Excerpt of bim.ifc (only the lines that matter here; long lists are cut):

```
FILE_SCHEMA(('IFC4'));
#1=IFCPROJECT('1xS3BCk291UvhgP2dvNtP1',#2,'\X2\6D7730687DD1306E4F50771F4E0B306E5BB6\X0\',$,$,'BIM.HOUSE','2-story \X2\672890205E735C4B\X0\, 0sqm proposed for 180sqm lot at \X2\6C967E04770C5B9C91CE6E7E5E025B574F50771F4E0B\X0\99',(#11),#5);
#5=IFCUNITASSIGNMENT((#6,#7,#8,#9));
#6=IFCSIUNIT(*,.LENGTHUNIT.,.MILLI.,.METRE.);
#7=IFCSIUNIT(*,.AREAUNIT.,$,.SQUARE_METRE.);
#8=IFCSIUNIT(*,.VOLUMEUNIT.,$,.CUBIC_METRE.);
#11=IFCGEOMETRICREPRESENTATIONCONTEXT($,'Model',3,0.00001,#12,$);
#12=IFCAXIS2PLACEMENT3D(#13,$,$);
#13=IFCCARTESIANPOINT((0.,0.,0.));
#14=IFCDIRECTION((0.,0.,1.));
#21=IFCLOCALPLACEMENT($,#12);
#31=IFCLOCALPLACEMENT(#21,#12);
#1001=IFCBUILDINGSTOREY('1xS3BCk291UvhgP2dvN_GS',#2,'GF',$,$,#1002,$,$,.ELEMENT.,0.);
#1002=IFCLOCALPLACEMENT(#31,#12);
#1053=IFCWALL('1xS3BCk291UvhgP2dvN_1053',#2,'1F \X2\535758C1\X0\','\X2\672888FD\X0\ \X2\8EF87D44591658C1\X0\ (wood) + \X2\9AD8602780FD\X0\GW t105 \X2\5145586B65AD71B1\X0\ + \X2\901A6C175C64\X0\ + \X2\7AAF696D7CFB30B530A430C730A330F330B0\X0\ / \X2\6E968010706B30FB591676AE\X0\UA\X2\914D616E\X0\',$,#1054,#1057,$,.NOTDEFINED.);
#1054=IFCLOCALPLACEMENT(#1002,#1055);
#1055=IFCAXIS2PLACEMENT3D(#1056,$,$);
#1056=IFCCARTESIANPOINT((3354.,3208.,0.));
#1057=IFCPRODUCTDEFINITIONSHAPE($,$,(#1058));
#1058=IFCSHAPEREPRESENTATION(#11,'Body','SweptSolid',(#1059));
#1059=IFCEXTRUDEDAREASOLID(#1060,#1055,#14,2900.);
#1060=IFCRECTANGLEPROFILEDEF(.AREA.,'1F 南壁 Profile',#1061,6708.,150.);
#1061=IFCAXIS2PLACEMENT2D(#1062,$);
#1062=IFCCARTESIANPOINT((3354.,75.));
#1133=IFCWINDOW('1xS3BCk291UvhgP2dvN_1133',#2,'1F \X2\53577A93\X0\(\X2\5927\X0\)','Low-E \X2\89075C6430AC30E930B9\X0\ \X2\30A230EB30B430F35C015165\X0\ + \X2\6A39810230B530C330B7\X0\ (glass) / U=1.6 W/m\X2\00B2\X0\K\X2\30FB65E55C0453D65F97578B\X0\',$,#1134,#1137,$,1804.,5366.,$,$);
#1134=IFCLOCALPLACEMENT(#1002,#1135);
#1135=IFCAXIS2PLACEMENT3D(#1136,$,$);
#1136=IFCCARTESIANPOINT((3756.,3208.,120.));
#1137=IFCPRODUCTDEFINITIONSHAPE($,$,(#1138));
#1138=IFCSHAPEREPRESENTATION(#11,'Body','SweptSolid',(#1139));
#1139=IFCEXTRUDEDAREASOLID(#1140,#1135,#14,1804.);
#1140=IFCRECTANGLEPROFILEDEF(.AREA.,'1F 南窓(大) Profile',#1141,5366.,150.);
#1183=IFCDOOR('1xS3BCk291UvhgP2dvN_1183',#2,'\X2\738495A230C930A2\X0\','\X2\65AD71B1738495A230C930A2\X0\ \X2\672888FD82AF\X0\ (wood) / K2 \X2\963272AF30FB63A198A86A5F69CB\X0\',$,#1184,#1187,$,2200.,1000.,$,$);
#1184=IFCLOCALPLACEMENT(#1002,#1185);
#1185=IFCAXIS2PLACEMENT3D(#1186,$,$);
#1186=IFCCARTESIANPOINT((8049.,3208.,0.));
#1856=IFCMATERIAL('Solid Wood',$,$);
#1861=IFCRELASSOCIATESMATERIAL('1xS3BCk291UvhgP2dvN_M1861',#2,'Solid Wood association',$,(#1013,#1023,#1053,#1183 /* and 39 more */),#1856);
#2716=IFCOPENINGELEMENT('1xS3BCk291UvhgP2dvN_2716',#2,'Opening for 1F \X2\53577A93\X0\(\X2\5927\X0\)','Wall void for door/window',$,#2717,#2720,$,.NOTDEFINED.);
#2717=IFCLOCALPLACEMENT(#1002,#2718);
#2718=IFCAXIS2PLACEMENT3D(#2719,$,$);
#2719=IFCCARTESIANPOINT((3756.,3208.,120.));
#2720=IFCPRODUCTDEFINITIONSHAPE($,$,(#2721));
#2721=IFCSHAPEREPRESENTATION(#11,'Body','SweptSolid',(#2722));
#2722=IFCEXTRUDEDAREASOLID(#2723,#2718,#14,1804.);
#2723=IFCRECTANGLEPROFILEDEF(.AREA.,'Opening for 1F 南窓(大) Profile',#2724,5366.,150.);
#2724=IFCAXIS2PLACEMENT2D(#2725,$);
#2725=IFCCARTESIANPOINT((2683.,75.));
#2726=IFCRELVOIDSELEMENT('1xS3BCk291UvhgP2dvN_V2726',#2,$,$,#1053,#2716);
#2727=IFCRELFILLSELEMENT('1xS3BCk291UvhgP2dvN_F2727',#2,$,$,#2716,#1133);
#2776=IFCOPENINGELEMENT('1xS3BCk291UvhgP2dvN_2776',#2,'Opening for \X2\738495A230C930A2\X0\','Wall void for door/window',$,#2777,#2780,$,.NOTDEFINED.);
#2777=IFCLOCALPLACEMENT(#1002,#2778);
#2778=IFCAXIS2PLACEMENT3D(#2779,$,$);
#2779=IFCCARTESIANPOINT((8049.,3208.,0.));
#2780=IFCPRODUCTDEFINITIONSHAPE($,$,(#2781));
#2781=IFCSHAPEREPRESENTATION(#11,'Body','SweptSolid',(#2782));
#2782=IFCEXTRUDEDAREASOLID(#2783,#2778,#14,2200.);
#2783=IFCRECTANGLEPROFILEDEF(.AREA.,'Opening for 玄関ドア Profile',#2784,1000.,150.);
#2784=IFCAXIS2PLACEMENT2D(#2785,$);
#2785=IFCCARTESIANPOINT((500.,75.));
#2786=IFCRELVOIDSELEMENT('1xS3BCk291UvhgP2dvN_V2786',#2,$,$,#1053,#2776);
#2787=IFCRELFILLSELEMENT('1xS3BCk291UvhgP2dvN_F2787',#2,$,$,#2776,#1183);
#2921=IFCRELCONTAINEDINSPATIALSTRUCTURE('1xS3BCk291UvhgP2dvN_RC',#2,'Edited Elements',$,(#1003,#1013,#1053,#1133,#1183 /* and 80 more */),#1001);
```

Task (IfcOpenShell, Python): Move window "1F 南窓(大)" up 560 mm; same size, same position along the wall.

```python
import numpy as np
import ifcopenshell
import ifcopenshell.api.geometry
import ifcopenshell.util.placement
import ifcopenshell.util.unit

model = ifcopenshell.open("bim.ifc")
unit_scale = ifcopenshell.util.unit.calculate_unit_scale(model)

window = model.by_guid("1xS3BCk291UvhgP2dvN_1133")
opening = window.FillsVoids[0].RelatingOpeningElement
dz = 560.0

shift = np.array([0.0, 0.0, dz])
# The window is not placed relative to its opening, so move both.
for product in (opening, window):
    matrix = ifcopenshell.util.placement.get_local_placement(product.ObjectPlacement)
    matrix[:3, 3] += shift
    ifcopenshell.api.geometry.edit_object_placement(model, product=product, matrix=matrix, is_si=False)

print(f"moved by {dz * unit_scale:+.3f} m")

model.write("bim_updated.ifc")
```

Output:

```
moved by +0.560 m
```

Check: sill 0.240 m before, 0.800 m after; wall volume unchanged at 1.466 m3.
